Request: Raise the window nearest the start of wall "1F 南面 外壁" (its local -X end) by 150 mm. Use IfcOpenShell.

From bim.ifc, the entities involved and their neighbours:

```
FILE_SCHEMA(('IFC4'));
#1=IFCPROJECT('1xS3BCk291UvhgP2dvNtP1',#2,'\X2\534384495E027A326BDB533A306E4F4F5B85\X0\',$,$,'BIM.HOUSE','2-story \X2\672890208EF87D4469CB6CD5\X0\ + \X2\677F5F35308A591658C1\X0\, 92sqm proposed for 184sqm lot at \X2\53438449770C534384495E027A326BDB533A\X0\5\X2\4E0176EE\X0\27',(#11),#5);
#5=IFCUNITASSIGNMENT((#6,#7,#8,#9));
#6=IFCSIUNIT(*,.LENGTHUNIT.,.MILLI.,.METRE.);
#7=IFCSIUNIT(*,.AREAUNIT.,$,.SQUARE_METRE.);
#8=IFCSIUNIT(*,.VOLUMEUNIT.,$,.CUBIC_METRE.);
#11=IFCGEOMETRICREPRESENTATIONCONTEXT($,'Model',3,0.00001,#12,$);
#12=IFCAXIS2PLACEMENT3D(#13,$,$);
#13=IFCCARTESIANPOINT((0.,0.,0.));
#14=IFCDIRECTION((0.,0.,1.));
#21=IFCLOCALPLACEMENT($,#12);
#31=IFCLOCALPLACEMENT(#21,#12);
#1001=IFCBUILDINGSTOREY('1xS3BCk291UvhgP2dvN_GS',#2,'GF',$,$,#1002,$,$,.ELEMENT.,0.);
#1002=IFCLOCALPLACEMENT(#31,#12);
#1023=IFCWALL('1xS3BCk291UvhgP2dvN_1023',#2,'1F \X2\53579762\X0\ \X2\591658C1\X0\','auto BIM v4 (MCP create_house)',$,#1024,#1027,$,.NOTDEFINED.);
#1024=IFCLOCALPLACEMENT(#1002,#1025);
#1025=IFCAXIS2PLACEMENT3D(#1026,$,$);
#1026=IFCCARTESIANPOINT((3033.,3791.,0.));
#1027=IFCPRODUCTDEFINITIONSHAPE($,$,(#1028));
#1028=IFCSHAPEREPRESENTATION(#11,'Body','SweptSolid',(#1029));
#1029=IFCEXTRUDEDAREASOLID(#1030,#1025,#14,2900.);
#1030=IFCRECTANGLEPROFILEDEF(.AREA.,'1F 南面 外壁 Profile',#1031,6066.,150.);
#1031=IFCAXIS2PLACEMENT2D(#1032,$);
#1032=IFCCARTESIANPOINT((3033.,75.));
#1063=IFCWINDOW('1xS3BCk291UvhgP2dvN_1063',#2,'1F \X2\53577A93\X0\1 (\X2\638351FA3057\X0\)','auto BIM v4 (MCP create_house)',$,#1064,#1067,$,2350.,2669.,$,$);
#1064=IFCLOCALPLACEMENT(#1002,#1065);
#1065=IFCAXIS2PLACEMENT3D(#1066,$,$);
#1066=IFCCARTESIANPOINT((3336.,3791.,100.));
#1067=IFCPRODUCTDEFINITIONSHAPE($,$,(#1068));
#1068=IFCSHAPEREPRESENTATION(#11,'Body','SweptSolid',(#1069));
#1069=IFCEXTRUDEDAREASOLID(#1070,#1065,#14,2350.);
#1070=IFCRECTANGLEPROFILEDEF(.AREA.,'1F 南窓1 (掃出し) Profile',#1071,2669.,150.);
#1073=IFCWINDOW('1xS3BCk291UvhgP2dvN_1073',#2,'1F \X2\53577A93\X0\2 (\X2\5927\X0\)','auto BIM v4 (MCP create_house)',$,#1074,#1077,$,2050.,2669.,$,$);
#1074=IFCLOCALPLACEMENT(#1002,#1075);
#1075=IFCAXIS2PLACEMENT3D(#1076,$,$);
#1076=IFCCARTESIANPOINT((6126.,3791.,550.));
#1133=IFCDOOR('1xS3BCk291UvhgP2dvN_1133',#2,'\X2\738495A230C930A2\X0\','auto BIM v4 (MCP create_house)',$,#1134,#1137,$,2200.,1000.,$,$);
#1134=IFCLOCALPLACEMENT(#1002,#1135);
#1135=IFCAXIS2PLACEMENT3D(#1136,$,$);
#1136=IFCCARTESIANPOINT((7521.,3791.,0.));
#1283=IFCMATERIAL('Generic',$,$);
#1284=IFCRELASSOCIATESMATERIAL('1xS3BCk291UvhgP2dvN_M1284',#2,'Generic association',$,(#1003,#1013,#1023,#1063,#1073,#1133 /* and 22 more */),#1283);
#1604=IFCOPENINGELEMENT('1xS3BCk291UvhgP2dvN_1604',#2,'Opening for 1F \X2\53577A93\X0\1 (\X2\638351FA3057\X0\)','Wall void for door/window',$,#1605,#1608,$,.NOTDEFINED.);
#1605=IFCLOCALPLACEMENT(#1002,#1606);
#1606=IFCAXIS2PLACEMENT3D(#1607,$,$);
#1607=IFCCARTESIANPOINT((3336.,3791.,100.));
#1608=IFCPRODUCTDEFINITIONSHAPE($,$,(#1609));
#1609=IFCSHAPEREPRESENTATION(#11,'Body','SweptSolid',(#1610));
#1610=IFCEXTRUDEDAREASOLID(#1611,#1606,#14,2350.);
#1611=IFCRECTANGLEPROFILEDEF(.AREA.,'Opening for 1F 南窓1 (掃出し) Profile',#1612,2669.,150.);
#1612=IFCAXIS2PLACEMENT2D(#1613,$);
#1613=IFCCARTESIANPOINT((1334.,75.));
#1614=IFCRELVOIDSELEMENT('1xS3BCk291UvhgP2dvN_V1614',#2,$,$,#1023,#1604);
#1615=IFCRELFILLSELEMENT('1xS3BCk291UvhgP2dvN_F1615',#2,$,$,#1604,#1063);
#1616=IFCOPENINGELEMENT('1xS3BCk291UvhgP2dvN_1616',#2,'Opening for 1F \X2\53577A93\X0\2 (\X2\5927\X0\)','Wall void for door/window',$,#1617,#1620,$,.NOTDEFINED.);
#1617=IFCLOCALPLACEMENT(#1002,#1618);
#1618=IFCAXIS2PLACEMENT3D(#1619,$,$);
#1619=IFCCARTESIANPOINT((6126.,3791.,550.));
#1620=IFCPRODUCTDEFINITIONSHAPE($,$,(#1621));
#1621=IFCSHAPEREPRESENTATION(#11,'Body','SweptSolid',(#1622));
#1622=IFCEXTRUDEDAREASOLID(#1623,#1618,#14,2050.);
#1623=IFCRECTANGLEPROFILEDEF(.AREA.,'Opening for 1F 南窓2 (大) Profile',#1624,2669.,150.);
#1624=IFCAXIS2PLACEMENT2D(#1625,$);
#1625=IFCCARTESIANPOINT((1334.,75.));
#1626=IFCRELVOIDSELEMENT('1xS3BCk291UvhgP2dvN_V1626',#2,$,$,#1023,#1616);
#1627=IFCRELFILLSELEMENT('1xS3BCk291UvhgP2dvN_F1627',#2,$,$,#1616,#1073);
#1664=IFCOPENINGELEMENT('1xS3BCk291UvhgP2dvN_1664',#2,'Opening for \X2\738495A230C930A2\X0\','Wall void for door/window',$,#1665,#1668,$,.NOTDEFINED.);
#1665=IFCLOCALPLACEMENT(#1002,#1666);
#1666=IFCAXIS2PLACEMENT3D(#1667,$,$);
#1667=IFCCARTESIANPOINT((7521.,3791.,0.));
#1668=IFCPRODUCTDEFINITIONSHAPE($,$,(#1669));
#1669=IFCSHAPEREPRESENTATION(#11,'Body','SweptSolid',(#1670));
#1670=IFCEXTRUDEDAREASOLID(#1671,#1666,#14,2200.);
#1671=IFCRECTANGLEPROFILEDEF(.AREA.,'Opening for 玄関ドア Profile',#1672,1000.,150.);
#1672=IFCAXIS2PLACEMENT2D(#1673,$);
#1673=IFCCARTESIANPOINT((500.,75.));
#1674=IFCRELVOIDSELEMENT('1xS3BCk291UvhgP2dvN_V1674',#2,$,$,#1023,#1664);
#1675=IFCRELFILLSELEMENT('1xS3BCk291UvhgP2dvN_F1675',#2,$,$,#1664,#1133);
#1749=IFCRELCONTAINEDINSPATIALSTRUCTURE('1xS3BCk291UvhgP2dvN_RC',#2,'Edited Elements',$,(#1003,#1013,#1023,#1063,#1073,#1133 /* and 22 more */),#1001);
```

```python
import numpy as np
import ifcopenshell
import ifcopenshell.api.geometry
import ifcopenshell.util.placement
import ifcopenshell.util.unit

model = ifcopenshell.open("bim.ifc")
unit_scale = ifcopenshell.util.unit.calculate_unit_scale(model)

window = model.by_guid("1xS3BCk291UvhgP2dvN_1063")
opening = window.FillsVoids[0].RelatingOpeningElement
dz = 0.15 / unit_scale

shift = np.array([0.0, 0.0, dz])
# The window is not placed relative to its opening, so move both.
for product in (opening, window):
    matrix = ifcopenshell.util.placement.get_local_placement(product.ObjectPlacement)
    matrix[:3, 3] += shift
    ifcopenshell.api.geometry.edit_object_placement(model, product=product, matrix=matrix, is_si=False)

print(f"moved by {dz * unit_scale:+.3f} m")

model.write("bim_edited.ifc")
```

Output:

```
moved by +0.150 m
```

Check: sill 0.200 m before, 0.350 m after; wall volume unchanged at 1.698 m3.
